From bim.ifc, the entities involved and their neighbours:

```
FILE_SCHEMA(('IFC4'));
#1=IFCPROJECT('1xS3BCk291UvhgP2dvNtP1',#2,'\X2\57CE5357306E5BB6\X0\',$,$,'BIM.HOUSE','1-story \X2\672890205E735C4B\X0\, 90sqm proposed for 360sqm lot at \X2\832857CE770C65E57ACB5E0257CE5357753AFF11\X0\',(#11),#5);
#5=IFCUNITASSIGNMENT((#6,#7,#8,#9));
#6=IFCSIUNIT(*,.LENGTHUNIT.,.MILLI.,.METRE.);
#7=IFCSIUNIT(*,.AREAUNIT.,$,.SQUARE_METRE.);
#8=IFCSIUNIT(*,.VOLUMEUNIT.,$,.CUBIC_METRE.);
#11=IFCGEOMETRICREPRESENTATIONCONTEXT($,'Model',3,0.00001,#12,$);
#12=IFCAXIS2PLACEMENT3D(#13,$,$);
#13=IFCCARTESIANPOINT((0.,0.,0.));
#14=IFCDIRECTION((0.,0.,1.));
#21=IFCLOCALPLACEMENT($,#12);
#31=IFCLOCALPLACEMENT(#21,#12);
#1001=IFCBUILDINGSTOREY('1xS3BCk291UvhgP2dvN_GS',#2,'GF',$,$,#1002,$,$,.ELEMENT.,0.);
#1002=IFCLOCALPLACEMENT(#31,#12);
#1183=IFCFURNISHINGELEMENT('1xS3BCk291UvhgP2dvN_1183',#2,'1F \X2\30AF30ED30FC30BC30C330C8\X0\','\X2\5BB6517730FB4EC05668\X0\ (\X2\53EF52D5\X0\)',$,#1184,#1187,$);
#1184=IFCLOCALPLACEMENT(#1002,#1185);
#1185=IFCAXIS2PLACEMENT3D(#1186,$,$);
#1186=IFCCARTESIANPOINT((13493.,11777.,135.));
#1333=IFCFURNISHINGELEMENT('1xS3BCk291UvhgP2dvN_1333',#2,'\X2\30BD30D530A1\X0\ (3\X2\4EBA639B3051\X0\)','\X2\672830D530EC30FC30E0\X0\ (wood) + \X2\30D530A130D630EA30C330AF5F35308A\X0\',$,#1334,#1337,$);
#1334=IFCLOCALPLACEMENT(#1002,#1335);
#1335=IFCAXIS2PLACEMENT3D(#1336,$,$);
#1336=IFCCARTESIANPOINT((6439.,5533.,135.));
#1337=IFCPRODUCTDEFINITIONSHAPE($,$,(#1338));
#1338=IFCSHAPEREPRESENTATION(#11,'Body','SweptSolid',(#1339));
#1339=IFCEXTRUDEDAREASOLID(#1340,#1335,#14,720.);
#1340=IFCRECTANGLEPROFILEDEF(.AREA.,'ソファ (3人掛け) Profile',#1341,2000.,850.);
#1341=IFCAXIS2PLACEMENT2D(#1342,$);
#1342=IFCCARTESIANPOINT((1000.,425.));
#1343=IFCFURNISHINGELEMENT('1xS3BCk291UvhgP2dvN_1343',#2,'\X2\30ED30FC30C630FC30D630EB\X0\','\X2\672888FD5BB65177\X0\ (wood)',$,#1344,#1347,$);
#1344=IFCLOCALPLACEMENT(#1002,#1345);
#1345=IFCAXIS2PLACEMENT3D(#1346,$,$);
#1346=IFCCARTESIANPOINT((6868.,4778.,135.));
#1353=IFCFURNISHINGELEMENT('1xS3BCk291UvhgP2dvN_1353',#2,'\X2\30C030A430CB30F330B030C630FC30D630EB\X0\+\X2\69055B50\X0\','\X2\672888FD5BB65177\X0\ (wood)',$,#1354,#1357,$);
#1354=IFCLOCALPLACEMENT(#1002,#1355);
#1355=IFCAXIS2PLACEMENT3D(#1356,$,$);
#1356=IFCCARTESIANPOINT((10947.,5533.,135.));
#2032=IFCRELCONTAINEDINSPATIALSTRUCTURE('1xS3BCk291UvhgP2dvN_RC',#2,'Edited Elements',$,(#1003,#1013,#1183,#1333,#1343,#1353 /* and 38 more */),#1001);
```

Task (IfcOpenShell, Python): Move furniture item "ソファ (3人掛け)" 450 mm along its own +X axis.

```python
import ifcopenshell
import ifcopenshell.api.geometry
import ifcopenshell.util.placement
import ifcopenshell.util.unit

model = ifcopenshell.open("bim.ifc")
unit_scale = ifcopenshell.util.unit.calculate_unit_scale(model)

item = model.by_guid("1xS3BCk291UvhgP2dvN_1333")
matrix = ifcopenshell.util.placement.get_local_placement(item.ObjectPlacement)
matrix[:3, 3] += matrix[:3, 0] * 0.45 / unit_scale
ifcopenshell.api.geometry.edit_object_placement(model, product=item, matrix=matrix, is_si=False)

print(ifcopenshell.util.placement.get_local_placement(item.ObjectPlacement).round(3) + 0.0)

model.write("bim_rev.ifc")
```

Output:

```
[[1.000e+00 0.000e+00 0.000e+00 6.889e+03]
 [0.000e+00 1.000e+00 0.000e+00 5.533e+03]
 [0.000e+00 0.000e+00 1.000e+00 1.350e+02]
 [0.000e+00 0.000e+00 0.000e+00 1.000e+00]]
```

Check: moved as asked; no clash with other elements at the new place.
